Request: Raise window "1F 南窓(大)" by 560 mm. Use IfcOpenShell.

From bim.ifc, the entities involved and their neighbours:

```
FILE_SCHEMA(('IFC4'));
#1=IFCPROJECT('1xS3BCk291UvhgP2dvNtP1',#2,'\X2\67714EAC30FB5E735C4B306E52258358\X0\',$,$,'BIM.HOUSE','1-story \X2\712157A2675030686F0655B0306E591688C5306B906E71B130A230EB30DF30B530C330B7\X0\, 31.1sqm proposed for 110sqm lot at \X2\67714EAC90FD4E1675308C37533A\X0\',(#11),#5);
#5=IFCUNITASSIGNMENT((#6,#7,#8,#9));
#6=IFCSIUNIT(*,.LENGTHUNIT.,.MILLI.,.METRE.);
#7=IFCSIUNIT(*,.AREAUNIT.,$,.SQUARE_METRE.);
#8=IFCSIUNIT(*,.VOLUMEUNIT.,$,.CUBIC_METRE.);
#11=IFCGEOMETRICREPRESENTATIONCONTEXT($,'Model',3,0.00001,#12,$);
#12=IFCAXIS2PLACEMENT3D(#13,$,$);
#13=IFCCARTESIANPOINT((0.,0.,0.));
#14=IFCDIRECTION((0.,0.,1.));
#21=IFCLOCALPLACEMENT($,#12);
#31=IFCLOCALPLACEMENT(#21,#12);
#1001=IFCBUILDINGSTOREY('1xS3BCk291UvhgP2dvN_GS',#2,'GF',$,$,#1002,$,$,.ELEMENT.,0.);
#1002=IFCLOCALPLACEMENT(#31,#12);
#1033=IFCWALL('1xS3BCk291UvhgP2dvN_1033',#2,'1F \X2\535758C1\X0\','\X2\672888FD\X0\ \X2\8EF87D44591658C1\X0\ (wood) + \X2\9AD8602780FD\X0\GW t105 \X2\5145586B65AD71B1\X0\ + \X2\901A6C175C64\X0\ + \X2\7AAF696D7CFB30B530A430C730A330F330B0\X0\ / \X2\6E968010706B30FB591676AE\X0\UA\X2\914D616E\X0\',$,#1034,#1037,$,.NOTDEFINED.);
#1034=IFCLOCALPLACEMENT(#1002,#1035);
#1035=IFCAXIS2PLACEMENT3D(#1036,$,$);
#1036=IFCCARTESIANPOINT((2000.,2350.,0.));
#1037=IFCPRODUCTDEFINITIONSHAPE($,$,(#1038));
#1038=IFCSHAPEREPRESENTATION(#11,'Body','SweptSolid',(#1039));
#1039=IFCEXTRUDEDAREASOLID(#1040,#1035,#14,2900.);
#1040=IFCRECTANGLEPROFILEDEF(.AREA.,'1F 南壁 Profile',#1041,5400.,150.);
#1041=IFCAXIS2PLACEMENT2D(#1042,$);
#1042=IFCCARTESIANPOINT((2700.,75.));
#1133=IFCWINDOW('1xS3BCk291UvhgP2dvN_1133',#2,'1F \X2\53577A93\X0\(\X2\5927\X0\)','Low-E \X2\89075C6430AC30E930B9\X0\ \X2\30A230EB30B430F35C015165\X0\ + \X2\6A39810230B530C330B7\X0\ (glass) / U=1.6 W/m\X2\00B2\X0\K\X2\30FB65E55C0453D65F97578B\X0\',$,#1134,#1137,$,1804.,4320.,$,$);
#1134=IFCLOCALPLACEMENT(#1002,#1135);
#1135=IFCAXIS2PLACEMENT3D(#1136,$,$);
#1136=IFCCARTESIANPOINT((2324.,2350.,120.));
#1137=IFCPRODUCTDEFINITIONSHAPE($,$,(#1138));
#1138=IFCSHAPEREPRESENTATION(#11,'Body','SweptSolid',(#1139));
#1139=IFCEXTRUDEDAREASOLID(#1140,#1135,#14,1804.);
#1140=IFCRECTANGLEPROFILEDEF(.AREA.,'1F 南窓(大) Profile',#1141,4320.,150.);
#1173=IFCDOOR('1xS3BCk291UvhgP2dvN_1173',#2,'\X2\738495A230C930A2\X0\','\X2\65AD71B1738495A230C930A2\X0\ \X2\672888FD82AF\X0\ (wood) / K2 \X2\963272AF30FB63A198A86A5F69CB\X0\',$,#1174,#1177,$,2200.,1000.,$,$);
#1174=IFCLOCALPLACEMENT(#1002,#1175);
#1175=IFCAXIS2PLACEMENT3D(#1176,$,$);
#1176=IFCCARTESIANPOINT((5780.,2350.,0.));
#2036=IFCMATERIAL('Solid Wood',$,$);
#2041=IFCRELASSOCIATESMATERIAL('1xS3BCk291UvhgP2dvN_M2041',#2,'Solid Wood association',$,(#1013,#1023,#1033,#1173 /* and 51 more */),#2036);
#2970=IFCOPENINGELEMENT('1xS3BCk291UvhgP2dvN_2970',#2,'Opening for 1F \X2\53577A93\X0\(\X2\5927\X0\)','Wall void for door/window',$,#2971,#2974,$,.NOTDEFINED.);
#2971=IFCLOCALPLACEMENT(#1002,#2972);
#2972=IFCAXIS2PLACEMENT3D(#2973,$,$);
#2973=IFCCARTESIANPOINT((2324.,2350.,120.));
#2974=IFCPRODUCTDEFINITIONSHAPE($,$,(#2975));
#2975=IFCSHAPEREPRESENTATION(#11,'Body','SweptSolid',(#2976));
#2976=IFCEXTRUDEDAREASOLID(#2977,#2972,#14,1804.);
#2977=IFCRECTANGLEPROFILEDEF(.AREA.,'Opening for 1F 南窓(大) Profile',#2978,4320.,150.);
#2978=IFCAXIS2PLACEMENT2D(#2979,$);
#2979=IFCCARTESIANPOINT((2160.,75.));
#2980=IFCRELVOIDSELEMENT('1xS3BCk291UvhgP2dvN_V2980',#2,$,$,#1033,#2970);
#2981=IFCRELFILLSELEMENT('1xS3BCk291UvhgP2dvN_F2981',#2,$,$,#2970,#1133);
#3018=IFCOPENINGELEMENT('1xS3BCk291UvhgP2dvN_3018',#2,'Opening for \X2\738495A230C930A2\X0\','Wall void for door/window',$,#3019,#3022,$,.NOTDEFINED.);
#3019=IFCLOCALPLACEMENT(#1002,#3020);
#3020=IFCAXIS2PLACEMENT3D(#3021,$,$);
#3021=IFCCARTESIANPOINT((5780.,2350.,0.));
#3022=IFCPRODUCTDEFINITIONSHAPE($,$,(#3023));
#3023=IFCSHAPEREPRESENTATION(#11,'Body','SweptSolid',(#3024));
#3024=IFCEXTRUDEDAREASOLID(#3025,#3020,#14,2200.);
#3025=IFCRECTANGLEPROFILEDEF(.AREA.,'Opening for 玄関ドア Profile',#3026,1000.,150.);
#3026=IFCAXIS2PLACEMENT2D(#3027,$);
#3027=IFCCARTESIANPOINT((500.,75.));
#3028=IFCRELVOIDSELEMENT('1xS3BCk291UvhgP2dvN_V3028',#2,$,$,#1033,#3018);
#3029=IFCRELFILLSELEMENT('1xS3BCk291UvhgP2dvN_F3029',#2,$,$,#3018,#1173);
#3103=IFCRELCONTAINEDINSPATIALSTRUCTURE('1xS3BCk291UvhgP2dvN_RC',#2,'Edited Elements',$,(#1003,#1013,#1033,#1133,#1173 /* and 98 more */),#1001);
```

```python
import numpy as np
import ifcopenshell
import ifcopenshell.api.geometry
import ifcopenshell.util.placement
import ifcopenshell.util.unit

model = ifcopenshell.open("bim.ifc")
unit_scale = ifcopenshell.util.unit.calculate_unit_scale(model)

window = model.by_id(1133)
opening = window.FillsVoids[0].RelatingOpeningElement
dz = 0.56 / unit_scale

shift = np.array([0.0, 0.0, dz])
# The window is not placed relative to its opening, so move both.
for product in (opening, window):
    matrix = ifcopenshell.util.placement.get_local_placement(product.ObjectPlacement)
    matrix[:3, 3] += shift
    ifcopenshell.api.geometry.edit_object_placement(model, product=product, matrix=matrix, is_si=False)

print(f"moved by {dz * unit_scale:+.3f} m")

model.write("bim_rev.ifc")
```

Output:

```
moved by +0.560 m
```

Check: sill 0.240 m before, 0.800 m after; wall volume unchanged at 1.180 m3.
